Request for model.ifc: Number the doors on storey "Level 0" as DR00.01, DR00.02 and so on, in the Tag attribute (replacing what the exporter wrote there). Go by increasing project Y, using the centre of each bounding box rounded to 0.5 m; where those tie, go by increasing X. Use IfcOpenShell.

First a look at what the model holds.

```python
import ifcopenshell
import ifcopenshell.util.element
import ifcopenshell.util.placement

model = ifcopenshell.open("model.ifc")
print(model.schema)
storey = next(s for s in model.by_type("IfcBuildingStorey") if s.Name == "Level 0")
doors = [e for e in ifcopenshell.util.element.get_decomposition(storey) if e.is_a("IfcDoor")]
for e in sorted(doors, key=lambda e: e.id()):
    origin = ifcopenshell.util.placement.get_local_placement(e.ObjectPlacement)[:3, 3]
    print(e.id(), e.Tag, e.Name, origin.round(2) + 0.0, sep=" | ")
```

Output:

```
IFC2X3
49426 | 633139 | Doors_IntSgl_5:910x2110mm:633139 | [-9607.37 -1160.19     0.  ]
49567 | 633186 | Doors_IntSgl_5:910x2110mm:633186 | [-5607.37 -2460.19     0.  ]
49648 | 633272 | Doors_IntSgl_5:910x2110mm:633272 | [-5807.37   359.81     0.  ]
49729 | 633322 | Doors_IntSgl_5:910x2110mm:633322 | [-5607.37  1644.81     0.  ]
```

```python
import ifcopenshell
import ifcopenshell.geom
import ifcopenshell.util.element
import ifcopenshell.util.shape

model = ifcopenshell.open("model.ifc")
settings = ifcopenshell.geom.settings()
settings.set("use-world-coords", True)


def centre(element):
    shape = ifcopenshell.geom.create_shape(settings, element)
    return ifcopenshell.util.shape.get_bbox_centroid(shape.geometry)


storey = next(s for s in model.by_type("IfcBuildingStorey") if s.Name == "Level 0")
doors = [e for e in ifcopenshell.util.element.get_decomposition(storey) if e.is_a("IfcDoor")]

# Insertion points can sit at a corner or the storey origin, so sort by the geometry (in metres).
centres = {e: centre(e) for e in doors}
doors.sort(key=lambda e: (round(centres[e][1] / 0.5), centres[e][0]))

for i, e in enumerate(doors, start=1):
    number = f"DR00.{i:02d}"
    e.Tag = number
    print(e.id(), number)

model.write("model_rev.ifc")
```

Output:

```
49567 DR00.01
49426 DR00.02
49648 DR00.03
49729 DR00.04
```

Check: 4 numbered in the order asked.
